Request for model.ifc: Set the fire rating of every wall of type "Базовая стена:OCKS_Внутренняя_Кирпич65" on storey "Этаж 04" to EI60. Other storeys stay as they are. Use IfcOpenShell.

First a look at what the model holds.

```python
import ifcopenshell
import ifcopenshell.util.element

model = ifcopenshell.open("model.ifc")
print(model.schema)
storey = next(s for s in model.by_type("IfcBuildingStorey") if s.Name == "Этаж 04")
walls = [e for e in ifcopenshell.util.element.get_decomposition(storey) if e.is_a("IfcWall")]
seen = {}
for e in walls:
    element_type = ifcopenshell.util.element.get_type(e)
    key = (element_type.Name if element_type != e and element_type else None, ifcopenshell.util.element.get_pset(e, "Pset_WallCommon", "FireRating"))
    seen[key] = seen.get(key, 0) + 1
for (name, value), count in sorted(seen.items(), key=str):
    print(count, "x", name, "|", value)
```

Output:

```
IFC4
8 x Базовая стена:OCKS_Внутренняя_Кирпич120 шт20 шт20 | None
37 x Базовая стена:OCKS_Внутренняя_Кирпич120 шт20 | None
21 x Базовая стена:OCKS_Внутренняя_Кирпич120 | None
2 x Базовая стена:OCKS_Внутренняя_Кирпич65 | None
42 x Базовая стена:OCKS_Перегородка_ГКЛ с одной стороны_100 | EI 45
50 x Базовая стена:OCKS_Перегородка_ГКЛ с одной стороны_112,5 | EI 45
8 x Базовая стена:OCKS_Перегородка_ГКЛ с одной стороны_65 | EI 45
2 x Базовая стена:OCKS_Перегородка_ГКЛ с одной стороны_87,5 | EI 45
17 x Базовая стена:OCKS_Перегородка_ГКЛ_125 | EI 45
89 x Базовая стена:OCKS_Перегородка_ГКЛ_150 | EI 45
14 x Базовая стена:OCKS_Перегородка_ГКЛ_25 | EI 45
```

```python
import ifcopenshell
import ifcopenshell.api.pset
import ifcopenshell.util.element

model = ifcopenshell.open("model.ifc")

storey = next(s for s in model.by_type("IfcBuildingStorey") if s.Name == "Этаж 04")
walls = [e for e in ifcopenshell.util.element.get_decomposition(storey) if e.is_a("IfcWall")]

count = 0
for e in walls:
    element_type = ifcopenshell.util.element.get_type(e)
    if element_type in (None, e) or element_type.Name != "Базовая стена:OCKS_Внутренняя_Кирпич65":
        continue
    # add_pset returns the element's existing set when there is one.
    pset = ifcopenshell.api.pset.add_pset(model, product=e, name="Pset_WallCommon")
    ifcopenshell.api.pset.edit_pset(model, pset=pset, properties={"FireRating": "EI60"})
    count += 1

print(count, "walls updated")

model.write("model_edited.ifc")
```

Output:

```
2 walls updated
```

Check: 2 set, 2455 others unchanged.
